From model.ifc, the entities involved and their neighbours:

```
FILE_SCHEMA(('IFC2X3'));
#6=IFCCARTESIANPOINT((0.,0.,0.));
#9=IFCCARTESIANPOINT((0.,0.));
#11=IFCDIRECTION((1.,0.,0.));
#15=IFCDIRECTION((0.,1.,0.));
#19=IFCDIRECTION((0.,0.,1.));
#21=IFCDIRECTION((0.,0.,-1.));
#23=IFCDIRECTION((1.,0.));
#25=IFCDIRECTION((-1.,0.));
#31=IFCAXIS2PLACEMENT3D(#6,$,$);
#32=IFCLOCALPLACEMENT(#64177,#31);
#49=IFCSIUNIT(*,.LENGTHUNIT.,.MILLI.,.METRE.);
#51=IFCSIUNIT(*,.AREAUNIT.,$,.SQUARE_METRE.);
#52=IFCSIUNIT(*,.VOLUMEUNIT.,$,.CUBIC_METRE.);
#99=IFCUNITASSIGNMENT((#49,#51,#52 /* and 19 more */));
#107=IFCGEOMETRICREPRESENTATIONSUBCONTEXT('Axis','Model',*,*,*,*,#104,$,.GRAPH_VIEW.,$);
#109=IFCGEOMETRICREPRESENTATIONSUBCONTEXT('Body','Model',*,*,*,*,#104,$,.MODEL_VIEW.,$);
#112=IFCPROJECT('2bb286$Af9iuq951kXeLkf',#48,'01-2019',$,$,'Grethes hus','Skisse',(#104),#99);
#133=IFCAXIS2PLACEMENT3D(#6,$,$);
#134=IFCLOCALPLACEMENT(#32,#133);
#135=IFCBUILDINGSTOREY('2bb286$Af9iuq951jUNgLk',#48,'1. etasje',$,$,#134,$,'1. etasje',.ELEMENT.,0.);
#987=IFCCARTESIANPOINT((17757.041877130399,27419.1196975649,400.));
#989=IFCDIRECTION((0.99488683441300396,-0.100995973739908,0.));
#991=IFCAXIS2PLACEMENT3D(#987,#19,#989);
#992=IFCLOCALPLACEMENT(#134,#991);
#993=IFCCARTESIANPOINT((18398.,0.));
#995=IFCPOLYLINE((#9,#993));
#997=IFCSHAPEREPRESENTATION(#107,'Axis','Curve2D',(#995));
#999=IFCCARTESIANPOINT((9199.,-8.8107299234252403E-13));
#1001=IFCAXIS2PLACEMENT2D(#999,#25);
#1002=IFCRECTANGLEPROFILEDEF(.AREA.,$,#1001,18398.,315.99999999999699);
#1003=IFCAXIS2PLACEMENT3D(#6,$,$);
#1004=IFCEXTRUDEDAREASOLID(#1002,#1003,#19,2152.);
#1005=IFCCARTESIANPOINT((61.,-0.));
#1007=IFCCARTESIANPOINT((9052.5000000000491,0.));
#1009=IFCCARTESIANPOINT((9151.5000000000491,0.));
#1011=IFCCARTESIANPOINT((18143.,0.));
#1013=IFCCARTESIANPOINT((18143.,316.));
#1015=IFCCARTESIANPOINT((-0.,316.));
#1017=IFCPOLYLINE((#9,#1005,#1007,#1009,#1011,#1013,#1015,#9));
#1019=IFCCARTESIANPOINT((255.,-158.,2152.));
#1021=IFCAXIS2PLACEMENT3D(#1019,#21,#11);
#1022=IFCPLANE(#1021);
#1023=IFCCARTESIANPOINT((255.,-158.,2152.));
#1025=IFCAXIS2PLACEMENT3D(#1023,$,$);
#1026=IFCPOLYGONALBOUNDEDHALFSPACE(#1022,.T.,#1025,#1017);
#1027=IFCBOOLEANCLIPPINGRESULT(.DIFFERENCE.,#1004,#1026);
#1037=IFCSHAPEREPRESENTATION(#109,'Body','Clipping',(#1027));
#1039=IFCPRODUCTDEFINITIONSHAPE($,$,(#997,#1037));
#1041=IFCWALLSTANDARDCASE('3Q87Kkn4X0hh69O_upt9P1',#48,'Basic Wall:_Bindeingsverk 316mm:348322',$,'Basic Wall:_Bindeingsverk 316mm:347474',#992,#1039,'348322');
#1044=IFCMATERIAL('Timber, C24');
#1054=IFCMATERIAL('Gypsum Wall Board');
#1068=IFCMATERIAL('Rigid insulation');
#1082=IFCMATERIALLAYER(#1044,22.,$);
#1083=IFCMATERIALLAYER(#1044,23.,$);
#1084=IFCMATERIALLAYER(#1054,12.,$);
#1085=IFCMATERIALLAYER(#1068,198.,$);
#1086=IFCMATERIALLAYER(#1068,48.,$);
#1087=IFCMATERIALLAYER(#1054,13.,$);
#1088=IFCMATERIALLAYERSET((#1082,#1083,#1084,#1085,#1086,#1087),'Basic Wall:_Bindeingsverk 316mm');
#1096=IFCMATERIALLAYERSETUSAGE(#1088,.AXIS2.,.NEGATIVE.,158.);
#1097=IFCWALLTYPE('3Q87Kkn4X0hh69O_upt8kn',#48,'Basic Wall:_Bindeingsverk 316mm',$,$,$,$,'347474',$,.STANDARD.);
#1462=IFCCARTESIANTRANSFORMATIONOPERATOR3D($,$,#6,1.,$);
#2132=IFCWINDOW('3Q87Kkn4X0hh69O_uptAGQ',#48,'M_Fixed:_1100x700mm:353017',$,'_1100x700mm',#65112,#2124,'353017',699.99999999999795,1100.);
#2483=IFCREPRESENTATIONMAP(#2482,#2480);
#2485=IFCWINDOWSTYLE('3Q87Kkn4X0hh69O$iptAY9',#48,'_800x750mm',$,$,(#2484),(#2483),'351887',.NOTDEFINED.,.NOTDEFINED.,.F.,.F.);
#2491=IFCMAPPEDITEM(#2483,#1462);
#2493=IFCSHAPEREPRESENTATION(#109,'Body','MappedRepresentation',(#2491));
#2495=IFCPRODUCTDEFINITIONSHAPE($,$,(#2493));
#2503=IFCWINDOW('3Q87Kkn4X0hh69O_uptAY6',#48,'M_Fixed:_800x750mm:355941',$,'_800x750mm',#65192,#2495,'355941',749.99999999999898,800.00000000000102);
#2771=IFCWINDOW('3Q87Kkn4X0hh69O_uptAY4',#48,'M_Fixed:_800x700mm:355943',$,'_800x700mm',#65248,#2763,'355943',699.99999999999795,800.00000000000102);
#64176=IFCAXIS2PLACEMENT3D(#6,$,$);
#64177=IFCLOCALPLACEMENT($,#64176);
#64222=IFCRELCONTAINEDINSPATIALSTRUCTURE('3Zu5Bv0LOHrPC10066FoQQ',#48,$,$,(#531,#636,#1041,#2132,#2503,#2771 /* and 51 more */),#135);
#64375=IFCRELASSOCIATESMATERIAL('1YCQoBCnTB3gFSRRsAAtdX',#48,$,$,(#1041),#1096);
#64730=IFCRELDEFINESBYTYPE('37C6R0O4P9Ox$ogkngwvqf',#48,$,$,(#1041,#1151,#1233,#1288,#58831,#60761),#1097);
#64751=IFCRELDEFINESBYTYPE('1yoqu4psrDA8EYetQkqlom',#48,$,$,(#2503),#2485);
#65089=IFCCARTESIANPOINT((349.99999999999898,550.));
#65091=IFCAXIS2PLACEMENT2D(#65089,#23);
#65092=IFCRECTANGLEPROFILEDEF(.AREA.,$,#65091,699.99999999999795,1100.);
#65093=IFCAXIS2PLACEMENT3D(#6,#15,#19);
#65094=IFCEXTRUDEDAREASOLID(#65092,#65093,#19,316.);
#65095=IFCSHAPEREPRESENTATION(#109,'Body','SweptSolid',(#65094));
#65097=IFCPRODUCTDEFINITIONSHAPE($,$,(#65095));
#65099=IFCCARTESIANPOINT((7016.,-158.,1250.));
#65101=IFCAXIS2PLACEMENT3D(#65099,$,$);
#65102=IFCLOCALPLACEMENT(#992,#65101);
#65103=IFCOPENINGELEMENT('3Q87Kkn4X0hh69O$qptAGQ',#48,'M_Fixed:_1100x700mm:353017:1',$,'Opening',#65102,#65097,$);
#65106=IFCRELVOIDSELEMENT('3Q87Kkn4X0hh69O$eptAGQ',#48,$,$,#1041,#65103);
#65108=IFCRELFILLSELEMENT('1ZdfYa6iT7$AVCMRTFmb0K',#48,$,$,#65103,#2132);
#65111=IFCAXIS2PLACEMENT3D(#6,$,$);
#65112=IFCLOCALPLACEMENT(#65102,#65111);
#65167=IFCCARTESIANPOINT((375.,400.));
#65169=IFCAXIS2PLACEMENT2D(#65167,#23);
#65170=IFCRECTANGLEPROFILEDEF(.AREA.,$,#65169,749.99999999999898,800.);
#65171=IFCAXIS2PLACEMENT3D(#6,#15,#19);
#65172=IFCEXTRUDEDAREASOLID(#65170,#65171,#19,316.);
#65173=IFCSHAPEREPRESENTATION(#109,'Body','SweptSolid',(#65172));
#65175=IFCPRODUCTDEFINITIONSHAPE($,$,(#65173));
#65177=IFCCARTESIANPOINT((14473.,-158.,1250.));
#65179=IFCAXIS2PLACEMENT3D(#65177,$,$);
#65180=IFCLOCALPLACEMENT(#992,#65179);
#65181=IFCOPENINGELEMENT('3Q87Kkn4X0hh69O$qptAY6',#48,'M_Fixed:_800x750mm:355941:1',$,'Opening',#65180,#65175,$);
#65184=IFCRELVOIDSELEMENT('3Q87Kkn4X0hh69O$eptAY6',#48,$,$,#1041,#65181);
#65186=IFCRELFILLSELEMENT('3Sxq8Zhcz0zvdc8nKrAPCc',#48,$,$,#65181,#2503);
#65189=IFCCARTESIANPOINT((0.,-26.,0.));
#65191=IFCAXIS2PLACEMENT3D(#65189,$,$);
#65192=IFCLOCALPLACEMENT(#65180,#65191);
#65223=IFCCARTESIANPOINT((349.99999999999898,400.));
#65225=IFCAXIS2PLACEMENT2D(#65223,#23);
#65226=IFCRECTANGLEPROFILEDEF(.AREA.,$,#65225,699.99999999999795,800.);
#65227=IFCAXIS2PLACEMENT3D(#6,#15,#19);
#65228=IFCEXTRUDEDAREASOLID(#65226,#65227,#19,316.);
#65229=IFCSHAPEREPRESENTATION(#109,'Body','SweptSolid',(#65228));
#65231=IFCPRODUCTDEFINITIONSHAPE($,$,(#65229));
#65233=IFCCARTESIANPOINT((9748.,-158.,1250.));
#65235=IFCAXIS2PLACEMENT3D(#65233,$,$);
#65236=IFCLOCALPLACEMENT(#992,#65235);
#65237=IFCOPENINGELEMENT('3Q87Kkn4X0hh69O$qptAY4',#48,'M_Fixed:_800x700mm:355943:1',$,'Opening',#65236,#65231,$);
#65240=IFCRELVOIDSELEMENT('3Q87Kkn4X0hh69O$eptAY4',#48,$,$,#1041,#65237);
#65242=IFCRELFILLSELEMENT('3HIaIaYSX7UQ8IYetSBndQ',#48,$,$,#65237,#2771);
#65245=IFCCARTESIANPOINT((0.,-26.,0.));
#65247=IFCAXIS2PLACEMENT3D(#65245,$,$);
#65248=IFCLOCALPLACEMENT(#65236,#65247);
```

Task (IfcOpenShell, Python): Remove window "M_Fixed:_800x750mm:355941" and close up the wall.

```python
import ifcopenshell
import ifcopenshell.api.feature
import ifcopenshell.api.root
import ifcopenshell.geom
import ifcopenshell.util.shape

model = ifcopenshell.open("model.ifc")
settings = ifcopenshell.geom.settings()


def volume(element):
    """Net volume in cubic metres, openings subtracted."""
    shape = ifcopenshell.geom.create_shape(settings, element)
    return ifcopenshell.util.shape.get_volume(shape.geometry)


window = model.by_guid("3Q87Kkn4X0hh69O_uptAY6")
opening = window.FillsVoids[0].RelatingOpeningElement
wall = opening.VoidsElements[0].RelatingBuildingElement
before = volume(wall)

ifcopenshell.api.root.remove_product(model, product=window)
ifcopenshell.api.feature.remove_feature(model, feature=opening)

after = volume(wall)

print(f"wall volume {before:.3f} -> {after:.3f} m3")

model.write("model_updated.ifc")
```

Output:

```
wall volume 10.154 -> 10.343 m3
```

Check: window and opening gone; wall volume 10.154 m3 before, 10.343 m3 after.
